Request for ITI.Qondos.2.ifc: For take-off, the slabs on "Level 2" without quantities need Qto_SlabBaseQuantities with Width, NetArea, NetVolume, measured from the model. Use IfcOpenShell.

First a look at what the model holds.

```python
import ifcopenshell
import ifcopenshell.util.element
import ifcopenshell.util.unit

model = ifcopenshell.open("ITI.Qondos.2.ifc")
print(model.schema)
for unit_type in ("LENGTHUNIT", "AREAUNIT", "VOLUMEUNIT"):
    print(unit_type, ifcopenshell.util.unit.calculate_unit_scale(model, unit_type))
storey = next(s for s in model.by_type("IfcBuildingStorey") if s.Name == "Level 2")
slabs = [e for e in ifcopenshell.util.element.get_decomposition(storey) if e.is_a("IfcSlab")]
for e in sorted(slabs, key=lambda e: e.id()):
    print(e.id(), e.is_a(), e.Name, list(ifcopenshell.util.element.get_psets(e, qtos_only=True)), sep=" | ")
```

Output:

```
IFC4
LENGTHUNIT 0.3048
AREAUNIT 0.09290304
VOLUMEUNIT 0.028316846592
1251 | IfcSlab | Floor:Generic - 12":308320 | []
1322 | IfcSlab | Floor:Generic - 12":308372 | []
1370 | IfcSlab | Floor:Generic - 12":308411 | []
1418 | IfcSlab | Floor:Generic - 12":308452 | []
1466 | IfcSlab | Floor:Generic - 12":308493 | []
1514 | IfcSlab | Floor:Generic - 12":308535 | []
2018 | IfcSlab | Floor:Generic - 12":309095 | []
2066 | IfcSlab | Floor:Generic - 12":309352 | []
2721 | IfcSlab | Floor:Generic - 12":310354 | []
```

```python
import ifcopenshell
import ifcopenshell.api.pset
import ifcopenshell.geom
import ifcopenshell.util.element
import ifcopenshell.util.shape
import ifcopenshell.util.unit

model = ifcopenshell.open("ITI.Qondos.2.ifc")
unit_scale = ifcopenshell.util.unit.calculate_unit_scale(model)
area_scale = ifcopenshell.util.unit.calculate_unit_scale(model, "AREAUNIT")
volume_scale = ifcopenshell.util.unit.calculate_unit_scale(model, "VOLUMEUNIT")
settings = ifcopenshell.geom.settings()

storey = next(s for s in model.by_type("IfcBuildingStorey") if s.Name == "Level 2")
slabs = [e for e in ifcopenshell.util.element.get_decomposition(storey) if e.is_a("IfcSlab")]

for e in sorted(slabs, key=lambda e: e.id()):
    if ifcopenshell.util.element.get_psets(e, qtos_only=True, should_inherit=False):
        continue
    # Geometry comes back in metres, in the element's own axes.
    shape = ifcopenshell.geom.create_shape(settings, e)
    values = {
        "Width": ifcopenshell.util.shape.get_z(shape.geometry) / unit_scale,
        "NetArea": ifcopenshell.util.shape.get_footprint_area(shape.geometry) / area_scale,
        "NetVolume": ifcopenshell.util.shape.get_volume(shape.geometry) / volume_scale,
    }
    qto = ifcopenshell.api.pset.add_qto(model, product=e, name="Qto_SlabBaseQuantities")
    ifcopenshell.api.pset.edit_qto(model, qto=qto, properties=values)
    print(e.id(), {k: round(v, 3) for k, v in values.items()})

model.write("ITI.Qondos.2_v2.ifc")
```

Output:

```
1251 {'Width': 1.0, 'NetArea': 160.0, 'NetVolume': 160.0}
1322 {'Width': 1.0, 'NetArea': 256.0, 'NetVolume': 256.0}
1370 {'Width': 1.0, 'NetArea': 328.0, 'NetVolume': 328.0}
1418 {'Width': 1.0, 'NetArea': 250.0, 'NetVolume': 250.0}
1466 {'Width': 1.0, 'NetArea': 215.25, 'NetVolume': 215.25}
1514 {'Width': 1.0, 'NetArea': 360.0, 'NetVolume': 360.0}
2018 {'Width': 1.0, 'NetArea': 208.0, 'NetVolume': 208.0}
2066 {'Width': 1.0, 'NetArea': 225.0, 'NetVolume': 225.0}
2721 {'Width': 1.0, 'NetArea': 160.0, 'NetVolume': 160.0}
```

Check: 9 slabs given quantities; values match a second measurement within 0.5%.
